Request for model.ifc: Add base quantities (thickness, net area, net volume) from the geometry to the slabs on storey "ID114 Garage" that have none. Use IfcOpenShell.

First a look at what the model holds.

```python
import ifcopenshell
import ifcopenshell.util.element
import ifcopenshell.util.unit

model = ifcopenshell.open("model.ifc")
print(model.schema)
for unit_type in ("LENGTHUNIT", "AREAUNIT", "VOLUMEUNIT"):
    print(unit_type, ifcopenshell.util.unit.calculate_unit_scale(model, unit_type))
storey = next(s for s in model.by_type("IfcBuildingStorey") if s.Name == "ID114 Garage")
slabs = [e for e in ifcopenshell.util.element.get_decomposition(storey) if e.is_a("IfcSlab")]
for e in sorted(slabs, key=lambda e: e.id()):
    print(e.id(), e.is_a(), e.Name, list(ifcopenshell.util.element.get_psets(e, qtos_only=True)), sep=" | ")
```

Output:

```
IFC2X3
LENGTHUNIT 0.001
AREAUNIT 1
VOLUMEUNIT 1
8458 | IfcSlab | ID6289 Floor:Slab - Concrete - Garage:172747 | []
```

```python
import ifcopenshell
import ifcopenshell.api.pset
import ifcopenshell.geom
import ifcopenshell.util.element
import ifcopenshell.util.shape
import ifcopenshell.util.unit

model = ifcopenshell.open("model.ifc")
unit_scale = ifcopenshell.util.unit.calculate_unit_scale(model)
area_scale = ifcopenshell.util.unit.calculate_unit_scale(model, "AREAUNIT")
volume_scale = ifcopenshell.util.unit.calculate_unit_scale(model, "VOLUMEUNIT")
settings = ifcopenshell.geom.settings()

storey = next(s for s in model.by_type("IfcBuildingStorey") if s.Name == "ID114 Garage")
slabs = [e for e in ifcopenshell.util.element.get_decomposition(storey) if e.is_a("IfcSlab")]

for e in sorted(slabs, key=lambda e: e.id()):
    if ifcopenshell.util.element.get_psets(e, qtos_only=True, should_inherit=False):
        continue
    # Geometry comes back in metres, in the element's own axes.
    shape = ifcopenshell.geom.create_shape(settings, e)
    values = {
        "Width": ifcopenshell.util.shape.get_z(shape.geometry) / unit_scale,
        "NetArea": ifcopenshell.util.shape.get_footprint_area(shape.geometry) / area_scale,
        "NetVolume": ifcopenshell.util.shape.get_volume(shape.geometry) / volume_scale,
    }
    qto = ifcopenshell.api.pset.add_qto(model, product=e, name="BaseQuantities")
    ifcopenshell.api.pset.edit_qto(model, qto=qto, properties=values)
    print(e.id(), {k: round(v, 3) for k, v in values.items()})

model.write("model_edited.ifc")
```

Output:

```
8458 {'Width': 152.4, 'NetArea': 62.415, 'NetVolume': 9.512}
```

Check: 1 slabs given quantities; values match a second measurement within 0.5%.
